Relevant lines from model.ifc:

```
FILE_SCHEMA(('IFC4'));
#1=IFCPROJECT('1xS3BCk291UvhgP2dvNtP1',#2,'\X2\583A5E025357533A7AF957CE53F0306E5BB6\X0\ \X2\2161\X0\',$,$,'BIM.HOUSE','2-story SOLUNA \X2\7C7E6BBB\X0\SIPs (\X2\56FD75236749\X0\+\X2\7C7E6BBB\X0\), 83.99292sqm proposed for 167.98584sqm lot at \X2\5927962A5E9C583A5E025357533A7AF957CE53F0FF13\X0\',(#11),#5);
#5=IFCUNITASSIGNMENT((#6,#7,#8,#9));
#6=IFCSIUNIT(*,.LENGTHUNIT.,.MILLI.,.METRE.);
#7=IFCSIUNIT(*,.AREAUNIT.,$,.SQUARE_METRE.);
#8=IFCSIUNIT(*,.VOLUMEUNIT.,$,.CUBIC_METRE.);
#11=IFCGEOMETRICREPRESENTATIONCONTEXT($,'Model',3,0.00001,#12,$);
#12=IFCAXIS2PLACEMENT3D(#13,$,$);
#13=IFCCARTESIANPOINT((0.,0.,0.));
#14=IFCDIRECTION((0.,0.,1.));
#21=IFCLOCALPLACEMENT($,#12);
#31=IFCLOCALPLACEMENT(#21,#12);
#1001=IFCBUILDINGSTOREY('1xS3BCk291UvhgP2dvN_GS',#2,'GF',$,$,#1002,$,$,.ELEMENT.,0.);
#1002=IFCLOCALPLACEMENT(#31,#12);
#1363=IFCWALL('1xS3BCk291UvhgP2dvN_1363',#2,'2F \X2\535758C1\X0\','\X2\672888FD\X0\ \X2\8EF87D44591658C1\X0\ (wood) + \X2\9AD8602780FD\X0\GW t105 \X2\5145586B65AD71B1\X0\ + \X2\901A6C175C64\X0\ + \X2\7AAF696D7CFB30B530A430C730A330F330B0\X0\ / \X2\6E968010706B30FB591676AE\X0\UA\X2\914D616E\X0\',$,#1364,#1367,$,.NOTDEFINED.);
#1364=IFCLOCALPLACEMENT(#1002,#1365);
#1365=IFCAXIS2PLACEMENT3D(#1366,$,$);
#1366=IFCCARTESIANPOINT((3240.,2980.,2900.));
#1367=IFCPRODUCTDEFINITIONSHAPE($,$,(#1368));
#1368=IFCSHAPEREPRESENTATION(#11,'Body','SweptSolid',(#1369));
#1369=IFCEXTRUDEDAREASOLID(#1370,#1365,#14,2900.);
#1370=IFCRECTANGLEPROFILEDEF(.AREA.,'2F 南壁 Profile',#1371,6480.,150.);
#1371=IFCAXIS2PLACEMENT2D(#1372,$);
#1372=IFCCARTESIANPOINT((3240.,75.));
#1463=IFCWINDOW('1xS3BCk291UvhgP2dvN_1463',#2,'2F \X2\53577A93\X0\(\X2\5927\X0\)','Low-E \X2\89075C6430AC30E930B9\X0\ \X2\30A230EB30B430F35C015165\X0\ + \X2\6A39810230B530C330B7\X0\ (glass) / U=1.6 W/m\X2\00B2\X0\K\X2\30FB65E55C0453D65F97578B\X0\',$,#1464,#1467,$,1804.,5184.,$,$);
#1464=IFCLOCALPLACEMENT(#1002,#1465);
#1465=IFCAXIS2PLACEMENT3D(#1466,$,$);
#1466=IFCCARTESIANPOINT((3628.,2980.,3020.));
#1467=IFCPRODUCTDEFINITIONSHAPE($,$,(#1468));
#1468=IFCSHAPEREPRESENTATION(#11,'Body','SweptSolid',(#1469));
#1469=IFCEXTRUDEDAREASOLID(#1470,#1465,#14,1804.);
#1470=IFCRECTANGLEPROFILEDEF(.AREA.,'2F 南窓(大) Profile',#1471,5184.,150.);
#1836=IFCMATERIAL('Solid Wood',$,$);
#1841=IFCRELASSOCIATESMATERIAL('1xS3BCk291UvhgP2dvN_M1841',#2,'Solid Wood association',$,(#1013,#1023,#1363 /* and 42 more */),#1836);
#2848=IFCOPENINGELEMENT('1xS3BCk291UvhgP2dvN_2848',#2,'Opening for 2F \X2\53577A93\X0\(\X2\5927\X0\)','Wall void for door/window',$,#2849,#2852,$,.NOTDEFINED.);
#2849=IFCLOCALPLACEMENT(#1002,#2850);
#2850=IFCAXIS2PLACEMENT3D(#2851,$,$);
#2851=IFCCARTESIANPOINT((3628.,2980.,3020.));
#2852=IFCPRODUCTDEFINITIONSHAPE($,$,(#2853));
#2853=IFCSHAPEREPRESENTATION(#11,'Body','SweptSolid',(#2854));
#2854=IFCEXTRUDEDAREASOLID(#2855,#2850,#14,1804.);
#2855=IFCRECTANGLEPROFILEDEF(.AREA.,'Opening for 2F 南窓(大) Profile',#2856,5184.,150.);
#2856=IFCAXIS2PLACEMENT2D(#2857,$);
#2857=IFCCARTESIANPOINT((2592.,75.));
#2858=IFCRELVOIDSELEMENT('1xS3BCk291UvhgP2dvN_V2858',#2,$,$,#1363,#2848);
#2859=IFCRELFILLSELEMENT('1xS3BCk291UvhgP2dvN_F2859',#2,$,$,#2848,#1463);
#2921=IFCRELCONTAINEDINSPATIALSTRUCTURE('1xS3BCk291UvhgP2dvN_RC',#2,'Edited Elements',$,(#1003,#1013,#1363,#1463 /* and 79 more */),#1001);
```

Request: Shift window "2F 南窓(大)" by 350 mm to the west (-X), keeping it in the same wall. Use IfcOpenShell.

```python
import ifcopenshell
import ifcopenshell.api.geometry
import ifcopenshell.util.placement

model = ifcopenshell.open("model.ifc")

window = model.by_guid("1xS3BCk291UvhgP2dvN_1463")
opening = window.FillsVoids[0].RelatingOpeningElement
wall = opening.VoidsElements[0].RelatingBuildingElement

wall_matrix = ifcopenshell.util.placement.get_local_placement(wall.ObjectPlacement)
shift = wall_matrix[:3, 0] * -350.0
before = ifcopenshell.util.placement.get_local_placement(window.ObjectPlacement)[:3, 3].copy()

# The window is not placed relative to its opening, so move both.
for product in (opening, window):
    matrix = ifcopenshell.util.placement.get_local_placement(product.ObjectPlacement)
    matrix[:3, 3] += shift
    ifcopenshell.api.geometry.edit_object_placement(model, product=product, matrix=matrix, is_si=False)

after = ifcopenshell.util.placement.get_local_placement(window.ObjectPlacement)[:3, 3]
print("window moved by", (after - before).round(3) + 0.0)

model.write("model-out.ifc")
```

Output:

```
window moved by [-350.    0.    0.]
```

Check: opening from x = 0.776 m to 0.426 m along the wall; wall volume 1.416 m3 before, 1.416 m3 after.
